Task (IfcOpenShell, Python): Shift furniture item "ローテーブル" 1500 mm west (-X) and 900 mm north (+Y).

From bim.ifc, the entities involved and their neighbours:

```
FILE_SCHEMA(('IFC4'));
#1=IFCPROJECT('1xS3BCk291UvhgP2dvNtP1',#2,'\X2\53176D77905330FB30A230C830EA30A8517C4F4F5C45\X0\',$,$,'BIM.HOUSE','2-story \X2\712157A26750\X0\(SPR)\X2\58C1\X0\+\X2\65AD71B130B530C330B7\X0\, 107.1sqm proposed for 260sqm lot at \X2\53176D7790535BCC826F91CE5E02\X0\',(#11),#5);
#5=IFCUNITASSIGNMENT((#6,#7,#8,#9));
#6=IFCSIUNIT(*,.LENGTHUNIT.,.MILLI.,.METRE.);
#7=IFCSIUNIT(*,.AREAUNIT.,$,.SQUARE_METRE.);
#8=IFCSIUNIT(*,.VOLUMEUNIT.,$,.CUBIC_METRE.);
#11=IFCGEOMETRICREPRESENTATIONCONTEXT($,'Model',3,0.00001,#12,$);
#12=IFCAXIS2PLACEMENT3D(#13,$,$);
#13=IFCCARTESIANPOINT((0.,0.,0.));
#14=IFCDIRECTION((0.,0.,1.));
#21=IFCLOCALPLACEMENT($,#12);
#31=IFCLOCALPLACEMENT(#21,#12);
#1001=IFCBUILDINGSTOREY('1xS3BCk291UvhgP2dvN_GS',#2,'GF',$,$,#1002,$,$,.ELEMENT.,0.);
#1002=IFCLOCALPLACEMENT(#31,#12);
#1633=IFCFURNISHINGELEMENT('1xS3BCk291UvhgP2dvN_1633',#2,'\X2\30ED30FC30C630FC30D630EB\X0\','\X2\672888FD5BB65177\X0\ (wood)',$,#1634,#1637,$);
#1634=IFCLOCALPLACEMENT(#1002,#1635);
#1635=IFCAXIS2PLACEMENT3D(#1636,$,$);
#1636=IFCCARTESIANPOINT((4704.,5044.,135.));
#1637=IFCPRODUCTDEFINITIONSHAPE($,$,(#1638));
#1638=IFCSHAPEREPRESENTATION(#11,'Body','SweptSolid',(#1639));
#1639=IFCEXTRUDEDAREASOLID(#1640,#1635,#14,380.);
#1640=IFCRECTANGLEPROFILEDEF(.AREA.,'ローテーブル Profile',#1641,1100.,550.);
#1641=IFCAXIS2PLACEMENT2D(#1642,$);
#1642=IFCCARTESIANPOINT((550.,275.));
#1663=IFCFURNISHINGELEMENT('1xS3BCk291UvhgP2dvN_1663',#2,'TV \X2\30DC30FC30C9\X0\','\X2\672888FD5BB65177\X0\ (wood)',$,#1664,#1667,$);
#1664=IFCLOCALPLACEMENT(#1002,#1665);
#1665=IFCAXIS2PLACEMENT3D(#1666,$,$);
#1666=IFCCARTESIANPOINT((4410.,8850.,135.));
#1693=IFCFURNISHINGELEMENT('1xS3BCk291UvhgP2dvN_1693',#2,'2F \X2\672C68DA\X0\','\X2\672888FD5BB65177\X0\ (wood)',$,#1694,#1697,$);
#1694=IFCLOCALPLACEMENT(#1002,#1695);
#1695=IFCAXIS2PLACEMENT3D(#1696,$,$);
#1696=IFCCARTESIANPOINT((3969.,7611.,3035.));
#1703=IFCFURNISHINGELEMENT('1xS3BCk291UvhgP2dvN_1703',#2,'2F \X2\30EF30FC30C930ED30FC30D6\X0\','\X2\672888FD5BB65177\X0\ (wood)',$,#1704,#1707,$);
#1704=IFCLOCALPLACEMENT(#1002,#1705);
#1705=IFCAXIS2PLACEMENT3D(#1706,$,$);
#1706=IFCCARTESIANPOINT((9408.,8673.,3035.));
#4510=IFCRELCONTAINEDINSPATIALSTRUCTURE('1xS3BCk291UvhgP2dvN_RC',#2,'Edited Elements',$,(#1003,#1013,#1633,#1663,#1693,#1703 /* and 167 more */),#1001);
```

```python
import ifcopenshell
import ifcopenshell.api.geometry
import ifcopenshell.util.placement
import ifcopenshell.util.unit

model = ifcopenshell.open("bim.ifc")
unit_scale = ifcopenshell.util.unit.calculate_unit_scale(model)

item = model.by_guid("1xS3BCk291UvhgP2dvN_1633")
matrix = ifcopenshell.util.placement.get_local_placement(item.ObjectPlacement)
matrix[0, 3] -= 1.5 / unit_scale
matrix[1, 3] += 0.9 / unit_scale
ifcopenshell.api.geometry.edit_object_placement(model, product=item, matrix=matrix, is_si=False)

print(ifcopenshell.util.placement.get_local_placement(item.ObjectPlacement).round(3) + 0.0)

model.write("bim_v2.ifc")
```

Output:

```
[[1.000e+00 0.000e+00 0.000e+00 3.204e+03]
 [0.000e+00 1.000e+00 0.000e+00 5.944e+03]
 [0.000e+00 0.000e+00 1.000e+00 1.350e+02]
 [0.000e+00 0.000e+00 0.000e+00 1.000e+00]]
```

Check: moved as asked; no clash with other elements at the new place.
